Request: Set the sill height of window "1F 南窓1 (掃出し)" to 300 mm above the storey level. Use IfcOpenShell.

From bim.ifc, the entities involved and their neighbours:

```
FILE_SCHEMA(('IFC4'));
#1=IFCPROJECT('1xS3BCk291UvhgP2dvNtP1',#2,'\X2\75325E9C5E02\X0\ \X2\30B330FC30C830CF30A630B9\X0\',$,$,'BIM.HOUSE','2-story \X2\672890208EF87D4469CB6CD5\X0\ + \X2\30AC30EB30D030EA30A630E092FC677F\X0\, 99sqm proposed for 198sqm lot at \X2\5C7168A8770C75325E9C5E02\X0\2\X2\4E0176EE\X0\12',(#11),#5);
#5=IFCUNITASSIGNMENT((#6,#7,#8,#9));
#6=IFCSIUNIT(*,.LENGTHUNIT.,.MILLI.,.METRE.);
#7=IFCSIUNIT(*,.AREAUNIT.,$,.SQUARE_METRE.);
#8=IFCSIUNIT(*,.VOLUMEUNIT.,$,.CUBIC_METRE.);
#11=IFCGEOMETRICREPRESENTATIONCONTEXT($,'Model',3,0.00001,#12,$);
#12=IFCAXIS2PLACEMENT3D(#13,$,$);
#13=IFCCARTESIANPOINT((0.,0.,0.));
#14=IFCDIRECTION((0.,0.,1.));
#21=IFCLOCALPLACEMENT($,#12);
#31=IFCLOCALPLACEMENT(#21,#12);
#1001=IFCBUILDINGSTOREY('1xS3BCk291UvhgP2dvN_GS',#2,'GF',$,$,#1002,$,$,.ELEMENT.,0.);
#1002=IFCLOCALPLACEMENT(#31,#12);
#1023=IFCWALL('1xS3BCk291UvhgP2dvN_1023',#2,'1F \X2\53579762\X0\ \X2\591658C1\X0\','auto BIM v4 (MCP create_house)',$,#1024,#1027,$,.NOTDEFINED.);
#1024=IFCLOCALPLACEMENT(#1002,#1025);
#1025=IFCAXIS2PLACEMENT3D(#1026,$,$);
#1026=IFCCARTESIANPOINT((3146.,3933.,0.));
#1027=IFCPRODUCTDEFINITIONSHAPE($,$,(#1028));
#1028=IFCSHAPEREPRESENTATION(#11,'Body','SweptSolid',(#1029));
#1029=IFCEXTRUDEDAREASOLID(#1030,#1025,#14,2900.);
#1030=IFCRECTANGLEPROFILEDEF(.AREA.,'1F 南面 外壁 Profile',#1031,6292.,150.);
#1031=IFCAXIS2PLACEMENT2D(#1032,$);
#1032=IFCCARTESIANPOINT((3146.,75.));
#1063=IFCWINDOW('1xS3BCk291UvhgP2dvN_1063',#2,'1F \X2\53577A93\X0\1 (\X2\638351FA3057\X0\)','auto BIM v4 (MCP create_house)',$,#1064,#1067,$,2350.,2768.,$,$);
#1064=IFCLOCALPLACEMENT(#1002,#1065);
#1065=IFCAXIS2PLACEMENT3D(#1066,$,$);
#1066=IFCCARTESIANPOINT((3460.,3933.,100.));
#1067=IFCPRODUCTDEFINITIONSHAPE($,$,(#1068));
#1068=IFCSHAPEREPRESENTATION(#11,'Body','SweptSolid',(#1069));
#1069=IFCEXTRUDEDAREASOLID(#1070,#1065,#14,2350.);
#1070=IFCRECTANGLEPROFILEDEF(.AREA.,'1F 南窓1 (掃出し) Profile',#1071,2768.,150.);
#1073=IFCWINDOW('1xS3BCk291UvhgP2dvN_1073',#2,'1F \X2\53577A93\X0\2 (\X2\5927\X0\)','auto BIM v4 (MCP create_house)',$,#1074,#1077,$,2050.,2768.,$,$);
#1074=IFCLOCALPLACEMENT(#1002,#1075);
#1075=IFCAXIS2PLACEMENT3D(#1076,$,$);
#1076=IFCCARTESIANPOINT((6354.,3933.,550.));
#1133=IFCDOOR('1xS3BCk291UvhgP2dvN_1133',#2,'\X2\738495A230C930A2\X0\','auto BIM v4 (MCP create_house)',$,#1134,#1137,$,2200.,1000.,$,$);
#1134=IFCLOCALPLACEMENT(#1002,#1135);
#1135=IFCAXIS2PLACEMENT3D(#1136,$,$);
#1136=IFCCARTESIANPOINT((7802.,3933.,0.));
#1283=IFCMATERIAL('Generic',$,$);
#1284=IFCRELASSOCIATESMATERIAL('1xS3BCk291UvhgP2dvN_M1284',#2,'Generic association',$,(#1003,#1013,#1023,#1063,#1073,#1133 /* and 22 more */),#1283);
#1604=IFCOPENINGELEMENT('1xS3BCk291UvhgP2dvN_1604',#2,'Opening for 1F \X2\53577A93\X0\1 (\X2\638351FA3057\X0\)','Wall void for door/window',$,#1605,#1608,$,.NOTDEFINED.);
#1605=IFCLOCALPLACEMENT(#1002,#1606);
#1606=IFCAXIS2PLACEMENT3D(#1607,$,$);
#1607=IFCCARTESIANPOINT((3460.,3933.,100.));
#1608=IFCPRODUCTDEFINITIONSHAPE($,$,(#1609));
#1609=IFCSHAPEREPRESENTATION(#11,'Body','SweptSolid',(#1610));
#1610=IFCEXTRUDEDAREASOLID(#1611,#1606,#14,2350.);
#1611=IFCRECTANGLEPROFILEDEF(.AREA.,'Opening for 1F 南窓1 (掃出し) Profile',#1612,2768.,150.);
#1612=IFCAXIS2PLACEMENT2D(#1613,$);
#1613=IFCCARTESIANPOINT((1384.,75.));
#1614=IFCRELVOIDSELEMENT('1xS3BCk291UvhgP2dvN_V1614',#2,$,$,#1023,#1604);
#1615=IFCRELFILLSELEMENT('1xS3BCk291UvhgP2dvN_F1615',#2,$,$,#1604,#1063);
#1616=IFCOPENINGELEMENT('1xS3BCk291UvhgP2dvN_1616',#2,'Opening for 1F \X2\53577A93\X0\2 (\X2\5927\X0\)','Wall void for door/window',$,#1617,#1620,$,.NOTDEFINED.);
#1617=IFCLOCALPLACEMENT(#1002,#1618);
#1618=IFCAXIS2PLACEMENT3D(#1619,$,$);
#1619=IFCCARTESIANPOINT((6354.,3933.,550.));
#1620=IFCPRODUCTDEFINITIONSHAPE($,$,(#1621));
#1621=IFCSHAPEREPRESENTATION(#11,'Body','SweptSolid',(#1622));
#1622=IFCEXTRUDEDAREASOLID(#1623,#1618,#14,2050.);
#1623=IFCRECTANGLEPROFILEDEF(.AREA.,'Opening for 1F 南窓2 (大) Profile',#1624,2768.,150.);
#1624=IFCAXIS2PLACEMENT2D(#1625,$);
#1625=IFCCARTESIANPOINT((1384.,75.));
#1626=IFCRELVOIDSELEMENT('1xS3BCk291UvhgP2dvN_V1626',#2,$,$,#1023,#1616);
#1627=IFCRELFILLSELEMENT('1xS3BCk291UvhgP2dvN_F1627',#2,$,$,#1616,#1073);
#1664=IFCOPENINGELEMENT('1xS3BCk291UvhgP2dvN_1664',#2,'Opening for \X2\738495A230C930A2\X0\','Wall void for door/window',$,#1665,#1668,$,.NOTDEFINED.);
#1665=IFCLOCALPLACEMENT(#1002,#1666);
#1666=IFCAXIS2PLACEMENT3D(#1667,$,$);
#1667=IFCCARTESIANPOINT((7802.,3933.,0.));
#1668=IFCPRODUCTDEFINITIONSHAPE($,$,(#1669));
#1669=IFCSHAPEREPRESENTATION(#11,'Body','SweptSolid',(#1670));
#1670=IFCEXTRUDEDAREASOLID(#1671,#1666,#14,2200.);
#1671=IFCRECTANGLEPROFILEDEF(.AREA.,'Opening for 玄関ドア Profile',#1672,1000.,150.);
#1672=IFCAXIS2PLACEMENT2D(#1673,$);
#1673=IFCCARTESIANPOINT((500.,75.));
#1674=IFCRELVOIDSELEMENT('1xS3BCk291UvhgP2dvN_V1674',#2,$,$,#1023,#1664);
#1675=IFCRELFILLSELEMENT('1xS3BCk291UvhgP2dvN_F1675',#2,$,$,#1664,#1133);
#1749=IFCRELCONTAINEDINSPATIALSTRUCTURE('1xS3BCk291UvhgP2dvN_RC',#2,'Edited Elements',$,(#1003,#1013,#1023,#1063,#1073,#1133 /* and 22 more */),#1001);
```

```python
import numpy as np
import ifcopenshell
import ifcopenshell.api.geometry
import ifcopenshell.geom
import ifcopenshell.util.element
import ifcopenshell.util.placement
import ifcopenshell.util.shape
import ifcopenshell.util.unit

model = ifcopenshell.open("bim.ifc")
unit_scale = ifcopenshell.util.unit.calculate_unit_scale(model)

window = model.by_guid("1xS3BCk291UvhgP2dvN_1063")
opening = window.FillsVoids[0].RelatingOpeningElement
storey = ifcopenshell.util.element.get_container(window, ifc_class="IfcBuildingStorey")
level = ifcopenshell.util.placement.get_local_placement(storey.ObjectPlacement)[2, 3]

# The opening's origin need not be at the sill, so measure its lowest point.
shape = ifcopenshell.geom.create_shape(ifcopenshell.geom.settings(), opening)
bottom = ifcopenshell.util.shape.get_shape_bottom_elevation(shape, shape.geometry) / unit_scale
dz = level + 0.3 / unit_scale - bottom

shift = np.array([0.0, 0.0, dz])
# The window is not placed relative to its opening, so move both.
for product in (opening, window):
    matrix = ifcopenshell.util.placement.get_local_placement(product.ObjectPlacement)
    matrix[:3, 3] += shift
    ifcopenshell.api.geometry.edit_object_placement(model, product=product, matrix=matrix, is_si=False)

print(f"moved by {dz * unit_scale:+.3f} m")

model.write("bim_v2.ifc")
```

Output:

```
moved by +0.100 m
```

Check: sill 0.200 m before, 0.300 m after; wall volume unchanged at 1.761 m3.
